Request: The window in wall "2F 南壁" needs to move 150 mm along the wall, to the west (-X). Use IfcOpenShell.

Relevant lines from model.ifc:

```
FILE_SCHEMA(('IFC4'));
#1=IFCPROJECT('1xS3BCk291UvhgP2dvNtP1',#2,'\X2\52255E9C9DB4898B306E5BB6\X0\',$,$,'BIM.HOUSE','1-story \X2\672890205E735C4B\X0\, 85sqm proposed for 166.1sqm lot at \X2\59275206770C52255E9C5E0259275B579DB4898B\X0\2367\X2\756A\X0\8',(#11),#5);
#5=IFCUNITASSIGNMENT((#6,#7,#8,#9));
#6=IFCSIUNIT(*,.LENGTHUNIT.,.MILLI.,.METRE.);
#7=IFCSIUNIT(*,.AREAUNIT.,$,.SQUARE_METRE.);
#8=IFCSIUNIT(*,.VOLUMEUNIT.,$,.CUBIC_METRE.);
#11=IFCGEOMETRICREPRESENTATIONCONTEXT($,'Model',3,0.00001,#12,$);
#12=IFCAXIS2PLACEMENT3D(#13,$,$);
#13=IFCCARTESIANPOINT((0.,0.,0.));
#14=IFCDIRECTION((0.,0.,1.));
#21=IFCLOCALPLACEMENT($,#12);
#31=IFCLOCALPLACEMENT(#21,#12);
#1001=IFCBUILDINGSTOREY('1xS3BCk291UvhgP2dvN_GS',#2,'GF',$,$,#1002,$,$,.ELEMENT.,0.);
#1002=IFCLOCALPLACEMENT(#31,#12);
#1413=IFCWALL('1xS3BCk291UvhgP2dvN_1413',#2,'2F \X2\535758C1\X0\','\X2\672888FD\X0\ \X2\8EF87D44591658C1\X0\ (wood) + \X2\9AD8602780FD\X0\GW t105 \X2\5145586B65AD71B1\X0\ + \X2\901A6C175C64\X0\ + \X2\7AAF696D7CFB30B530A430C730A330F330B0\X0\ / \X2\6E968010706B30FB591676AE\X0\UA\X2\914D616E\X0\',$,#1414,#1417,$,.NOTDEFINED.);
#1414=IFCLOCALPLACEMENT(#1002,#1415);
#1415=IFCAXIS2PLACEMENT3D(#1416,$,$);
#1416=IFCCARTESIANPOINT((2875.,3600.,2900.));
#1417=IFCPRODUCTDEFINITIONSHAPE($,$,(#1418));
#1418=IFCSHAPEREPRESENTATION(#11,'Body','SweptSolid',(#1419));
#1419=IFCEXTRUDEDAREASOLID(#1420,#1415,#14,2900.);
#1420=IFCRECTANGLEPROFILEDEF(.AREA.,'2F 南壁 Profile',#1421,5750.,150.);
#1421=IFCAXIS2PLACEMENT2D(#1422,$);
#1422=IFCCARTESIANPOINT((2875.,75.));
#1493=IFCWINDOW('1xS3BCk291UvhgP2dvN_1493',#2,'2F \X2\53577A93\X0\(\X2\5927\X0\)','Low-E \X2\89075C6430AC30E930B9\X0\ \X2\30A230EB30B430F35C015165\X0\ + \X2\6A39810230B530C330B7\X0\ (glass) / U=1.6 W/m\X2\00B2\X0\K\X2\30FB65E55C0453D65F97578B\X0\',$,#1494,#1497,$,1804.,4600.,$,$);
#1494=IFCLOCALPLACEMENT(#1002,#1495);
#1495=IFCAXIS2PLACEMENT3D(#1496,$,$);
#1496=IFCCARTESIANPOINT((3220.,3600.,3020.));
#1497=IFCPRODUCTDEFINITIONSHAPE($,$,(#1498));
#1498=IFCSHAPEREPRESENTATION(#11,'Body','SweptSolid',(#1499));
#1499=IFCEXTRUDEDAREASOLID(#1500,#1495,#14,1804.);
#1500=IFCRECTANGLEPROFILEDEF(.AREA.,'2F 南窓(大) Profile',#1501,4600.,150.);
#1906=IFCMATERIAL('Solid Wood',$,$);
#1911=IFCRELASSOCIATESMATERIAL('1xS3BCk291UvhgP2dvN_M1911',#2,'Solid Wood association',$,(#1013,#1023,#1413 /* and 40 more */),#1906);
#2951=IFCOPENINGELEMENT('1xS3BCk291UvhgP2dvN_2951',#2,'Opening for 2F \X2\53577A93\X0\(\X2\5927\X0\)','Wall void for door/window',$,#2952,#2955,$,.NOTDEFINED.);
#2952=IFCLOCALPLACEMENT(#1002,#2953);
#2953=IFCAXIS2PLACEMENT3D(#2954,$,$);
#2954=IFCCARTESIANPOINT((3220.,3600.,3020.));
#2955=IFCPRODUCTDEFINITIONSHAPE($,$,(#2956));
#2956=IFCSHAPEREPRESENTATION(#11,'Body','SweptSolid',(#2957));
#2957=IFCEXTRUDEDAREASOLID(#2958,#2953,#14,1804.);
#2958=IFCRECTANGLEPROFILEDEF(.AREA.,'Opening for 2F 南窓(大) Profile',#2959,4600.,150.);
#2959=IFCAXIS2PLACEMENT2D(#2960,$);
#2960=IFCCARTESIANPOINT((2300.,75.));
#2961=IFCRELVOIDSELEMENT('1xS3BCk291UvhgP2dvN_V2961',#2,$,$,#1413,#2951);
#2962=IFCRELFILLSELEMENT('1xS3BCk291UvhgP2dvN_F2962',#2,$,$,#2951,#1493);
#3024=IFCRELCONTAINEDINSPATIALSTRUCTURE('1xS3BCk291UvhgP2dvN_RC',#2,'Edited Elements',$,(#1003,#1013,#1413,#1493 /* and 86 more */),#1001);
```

```python
import ifcopenshell
import ifcopenshell.api.geometry
import ifcopenshell.util.placement
import ifcopenshell.util.unit

model = ifcopenshell.open("model.ifc")
unit_scale = ifcopenshell.util.unit.calculate_unit_scale(model)

window = model.by_guid("1xS3BCk291UvhgP2dvN_1493")
opening = window.FillsVoids[0].RelatingOpeningElement
wall = opening.VoidsElements[0].RelatingBuildingElement

wall_matrix = ifcopenshell.util.placement.get_local_placement(wall.ObjectPlacement)
shift = wall_matrix[:3, 0] * -0.15 / unit_scale
before = ifcopenshell.util.placement.get_local_placement(window.ObjectPlacement)[:3, 3].copy()

# The window is not placed relative to its opening, so move both.
for product in (opening, window):
    matrix = ifcopenshell.util.placement.get_local_placement(product.ObjectPlacement)
    matrix[:3, 3] += shift
    ifcopenshell.api.geometry.edit_object_placement(model, product=product, matrix=matrix, is_si=False)

after = ifcopenshell.util.placement.get_local_placement(window.ObjectPlacement)[:3, 3]
print("window moved by", (after - before).round(3) + 0.0)

model.write("model_updated.ifc")
```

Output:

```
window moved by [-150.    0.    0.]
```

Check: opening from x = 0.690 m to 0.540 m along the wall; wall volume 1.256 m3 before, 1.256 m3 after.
